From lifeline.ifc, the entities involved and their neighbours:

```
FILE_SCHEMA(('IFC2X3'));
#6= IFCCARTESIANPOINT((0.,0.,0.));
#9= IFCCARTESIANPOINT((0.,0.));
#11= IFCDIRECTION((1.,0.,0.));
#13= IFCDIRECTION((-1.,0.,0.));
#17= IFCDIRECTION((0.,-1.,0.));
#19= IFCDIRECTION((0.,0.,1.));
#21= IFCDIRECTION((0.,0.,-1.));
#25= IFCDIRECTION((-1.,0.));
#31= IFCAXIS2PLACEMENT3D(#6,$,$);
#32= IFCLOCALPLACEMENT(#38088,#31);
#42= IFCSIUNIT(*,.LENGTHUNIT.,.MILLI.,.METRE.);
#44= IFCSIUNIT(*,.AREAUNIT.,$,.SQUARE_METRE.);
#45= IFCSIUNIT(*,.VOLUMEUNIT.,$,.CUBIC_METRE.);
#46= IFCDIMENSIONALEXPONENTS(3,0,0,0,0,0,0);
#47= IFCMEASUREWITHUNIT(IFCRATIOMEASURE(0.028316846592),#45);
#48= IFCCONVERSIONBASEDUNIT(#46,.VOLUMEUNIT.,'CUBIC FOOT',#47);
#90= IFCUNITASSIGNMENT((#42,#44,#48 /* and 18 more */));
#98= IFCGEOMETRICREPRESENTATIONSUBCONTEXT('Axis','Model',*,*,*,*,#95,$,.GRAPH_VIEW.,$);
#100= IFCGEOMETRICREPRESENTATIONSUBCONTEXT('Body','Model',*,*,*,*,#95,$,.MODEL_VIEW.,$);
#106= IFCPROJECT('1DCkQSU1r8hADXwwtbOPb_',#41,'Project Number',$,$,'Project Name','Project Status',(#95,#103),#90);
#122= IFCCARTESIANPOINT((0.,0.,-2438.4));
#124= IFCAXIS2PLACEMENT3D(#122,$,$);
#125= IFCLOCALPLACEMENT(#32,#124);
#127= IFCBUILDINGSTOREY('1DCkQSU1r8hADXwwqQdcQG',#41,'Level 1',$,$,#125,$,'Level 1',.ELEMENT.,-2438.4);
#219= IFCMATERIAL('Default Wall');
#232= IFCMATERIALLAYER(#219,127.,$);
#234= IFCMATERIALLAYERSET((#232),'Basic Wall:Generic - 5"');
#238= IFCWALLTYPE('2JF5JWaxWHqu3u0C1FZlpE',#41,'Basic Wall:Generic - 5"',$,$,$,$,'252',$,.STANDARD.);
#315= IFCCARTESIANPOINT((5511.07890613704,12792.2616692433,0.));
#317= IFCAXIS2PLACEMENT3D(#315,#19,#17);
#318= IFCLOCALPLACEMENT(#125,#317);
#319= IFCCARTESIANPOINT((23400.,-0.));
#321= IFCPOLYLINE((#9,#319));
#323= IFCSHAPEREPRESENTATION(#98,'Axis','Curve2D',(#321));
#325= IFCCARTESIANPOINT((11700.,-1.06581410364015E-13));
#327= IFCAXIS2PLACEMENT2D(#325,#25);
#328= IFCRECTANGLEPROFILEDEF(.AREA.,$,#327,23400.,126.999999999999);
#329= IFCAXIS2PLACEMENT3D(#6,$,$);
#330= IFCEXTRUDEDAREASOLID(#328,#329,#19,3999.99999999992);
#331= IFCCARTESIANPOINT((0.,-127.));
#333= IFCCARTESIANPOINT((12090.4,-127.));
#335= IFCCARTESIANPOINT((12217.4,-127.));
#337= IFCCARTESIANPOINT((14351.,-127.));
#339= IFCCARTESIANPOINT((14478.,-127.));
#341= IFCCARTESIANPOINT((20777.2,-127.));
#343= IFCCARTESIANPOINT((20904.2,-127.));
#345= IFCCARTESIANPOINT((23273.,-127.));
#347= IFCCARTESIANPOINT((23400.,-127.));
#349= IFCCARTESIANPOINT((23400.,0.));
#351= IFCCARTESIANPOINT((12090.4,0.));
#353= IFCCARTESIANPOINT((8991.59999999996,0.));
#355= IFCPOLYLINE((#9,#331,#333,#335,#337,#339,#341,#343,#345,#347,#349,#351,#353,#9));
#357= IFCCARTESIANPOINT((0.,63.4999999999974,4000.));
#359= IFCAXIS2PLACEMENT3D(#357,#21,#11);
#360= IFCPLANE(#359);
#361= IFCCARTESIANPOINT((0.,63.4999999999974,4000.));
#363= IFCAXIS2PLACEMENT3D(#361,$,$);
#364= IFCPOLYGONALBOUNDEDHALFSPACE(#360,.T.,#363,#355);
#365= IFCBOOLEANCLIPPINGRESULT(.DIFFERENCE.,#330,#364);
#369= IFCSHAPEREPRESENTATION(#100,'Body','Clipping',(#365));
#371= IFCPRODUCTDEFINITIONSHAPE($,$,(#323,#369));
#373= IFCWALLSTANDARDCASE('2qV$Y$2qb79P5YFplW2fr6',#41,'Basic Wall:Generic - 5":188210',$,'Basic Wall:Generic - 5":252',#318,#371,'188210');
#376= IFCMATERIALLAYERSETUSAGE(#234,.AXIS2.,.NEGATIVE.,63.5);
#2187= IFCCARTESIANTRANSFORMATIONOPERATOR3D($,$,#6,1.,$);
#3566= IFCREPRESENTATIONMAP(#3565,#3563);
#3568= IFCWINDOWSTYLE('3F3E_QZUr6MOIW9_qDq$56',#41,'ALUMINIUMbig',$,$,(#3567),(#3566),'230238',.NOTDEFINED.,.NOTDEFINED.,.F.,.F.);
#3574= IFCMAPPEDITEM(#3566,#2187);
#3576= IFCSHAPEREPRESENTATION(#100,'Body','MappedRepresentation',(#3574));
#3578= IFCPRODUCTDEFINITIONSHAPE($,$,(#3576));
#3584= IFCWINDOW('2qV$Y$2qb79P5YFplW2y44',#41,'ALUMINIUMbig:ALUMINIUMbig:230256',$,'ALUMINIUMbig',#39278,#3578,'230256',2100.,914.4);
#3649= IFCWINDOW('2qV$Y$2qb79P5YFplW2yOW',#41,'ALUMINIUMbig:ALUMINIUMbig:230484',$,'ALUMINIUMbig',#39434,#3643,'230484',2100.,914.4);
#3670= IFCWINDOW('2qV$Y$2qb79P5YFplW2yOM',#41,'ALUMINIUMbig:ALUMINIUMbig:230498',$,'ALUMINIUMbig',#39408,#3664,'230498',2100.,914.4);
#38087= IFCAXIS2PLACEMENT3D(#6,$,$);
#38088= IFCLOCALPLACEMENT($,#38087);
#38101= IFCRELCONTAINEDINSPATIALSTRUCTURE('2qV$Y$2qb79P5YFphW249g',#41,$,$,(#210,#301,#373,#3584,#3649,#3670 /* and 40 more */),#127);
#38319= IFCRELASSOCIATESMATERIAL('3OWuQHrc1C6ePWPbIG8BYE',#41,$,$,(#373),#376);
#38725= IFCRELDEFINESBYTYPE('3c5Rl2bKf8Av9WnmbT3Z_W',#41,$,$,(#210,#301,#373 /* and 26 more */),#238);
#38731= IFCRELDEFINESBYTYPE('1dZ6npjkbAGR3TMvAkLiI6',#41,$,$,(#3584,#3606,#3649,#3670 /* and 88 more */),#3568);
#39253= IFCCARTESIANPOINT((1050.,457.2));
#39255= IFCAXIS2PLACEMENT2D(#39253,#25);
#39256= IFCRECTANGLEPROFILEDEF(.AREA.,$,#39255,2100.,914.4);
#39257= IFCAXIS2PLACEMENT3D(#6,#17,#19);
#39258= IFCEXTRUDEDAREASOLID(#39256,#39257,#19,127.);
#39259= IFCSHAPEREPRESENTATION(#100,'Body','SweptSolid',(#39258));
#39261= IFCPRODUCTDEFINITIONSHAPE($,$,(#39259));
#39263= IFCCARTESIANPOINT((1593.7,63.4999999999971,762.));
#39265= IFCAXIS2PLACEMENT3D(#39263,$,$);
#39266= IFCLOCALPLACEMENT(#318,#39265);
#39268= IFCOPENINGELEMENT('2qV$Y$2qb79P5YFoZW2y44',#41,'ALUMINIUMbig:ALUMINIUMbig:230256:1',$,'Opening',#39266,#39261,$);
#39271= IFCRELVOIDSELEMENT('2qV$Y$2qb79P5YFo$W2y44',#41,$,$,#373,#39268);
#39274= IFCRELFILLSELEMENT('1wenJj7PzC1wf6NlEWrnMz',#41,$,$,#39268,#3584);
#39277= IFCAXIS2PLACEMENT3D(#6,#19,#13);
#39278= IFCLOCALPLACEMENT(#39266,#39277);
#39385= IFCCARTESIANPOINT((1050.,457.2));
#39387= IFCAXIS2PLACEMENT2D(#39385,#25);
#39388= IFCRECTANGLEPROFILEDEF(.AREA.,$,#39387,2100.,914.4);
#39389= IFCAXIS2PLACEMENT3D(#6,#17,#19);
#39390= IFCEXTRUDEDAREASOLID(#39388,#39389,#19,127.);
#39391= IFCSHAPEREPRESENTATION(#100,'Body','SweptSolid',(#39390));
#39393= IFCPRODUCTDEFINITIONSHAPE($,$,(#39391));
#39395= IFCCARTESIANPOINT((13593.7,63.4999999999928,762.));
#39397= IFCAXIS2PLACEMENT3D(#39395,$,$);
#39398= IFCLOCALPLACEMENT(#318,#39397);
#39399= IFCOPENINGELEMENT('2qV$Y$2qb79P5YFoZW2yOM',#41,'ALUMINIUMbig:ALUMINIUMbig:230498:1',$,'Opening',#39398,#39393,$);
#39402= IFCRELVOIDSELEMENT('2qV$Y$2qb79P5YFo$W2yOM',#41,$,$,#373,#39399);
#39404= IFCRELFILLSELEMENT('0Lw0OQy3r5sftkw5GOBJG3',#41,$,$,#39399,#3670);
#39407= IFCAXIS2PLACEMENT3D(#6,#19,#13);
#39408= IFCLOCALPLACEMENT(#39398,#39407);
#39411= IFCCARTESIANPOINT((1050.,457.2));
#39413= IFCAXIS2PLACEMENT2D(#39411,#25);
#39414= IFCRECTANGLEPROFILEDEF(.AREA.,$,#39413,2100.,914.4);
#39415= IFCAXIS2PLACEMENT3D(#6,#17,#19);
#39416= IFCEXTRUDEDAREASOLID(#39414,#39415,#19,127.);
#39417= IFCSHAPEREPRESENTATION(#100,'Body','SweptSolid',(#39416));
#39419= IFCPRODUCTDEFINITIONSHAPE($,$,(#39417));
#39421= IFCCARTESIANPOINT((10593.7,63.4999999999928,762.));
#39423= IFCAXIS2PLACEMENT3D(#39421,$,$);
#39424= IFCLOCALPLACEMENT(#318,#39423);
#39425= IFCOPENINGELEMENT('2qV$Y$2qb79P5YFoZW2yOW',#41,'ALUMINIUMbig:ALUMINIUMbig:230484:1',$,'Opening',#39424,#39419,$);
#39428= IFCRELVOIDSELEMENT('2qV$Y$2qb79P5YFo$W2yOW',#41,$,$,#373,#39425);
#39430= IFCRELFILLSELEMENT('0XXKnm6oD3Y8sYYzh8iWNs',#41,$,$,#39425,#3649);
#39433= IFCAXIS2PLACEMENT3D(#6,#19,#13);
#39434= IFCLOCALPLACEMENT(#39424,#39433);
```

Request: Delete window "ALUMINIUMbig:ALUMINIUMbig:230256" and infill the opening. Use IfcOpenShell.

```python
import ifcopenshell
import ifcopenshell.api.feature
import ifcopenshell.api.root
import ifcopenshell.geom
import ifcopenshell.util.shape

model = ifcopenshell.open("lifeline.ifc")
settings = ifcopenshell.geom.settings()


def volume(element):
    """Net volume in cubic metres, openings subtracted."""
    shape = ifcopenshell.geom.create_shape(settings, element)
    return ifcopenshell.util.shape.get_volume(shape.geometry)


window = model.by_guid("2qV$Y$2qb79P5YFplW2y44")
opening = window.FillsVoids[0].RelatingOpeningElement
wall = opening.VoidsElements[0].RelatingBuildingElement
before = volume(wall)

ifcopenshell.api.root.remove_product(model, product=window)
ifcopenshell.api.feature.remove_feature(model, feature=opening)

after = volume(wall)

print(f"wall volume {before:.3f} -> {after:.3f} m3")

model.write("lifeline_rev.ifc")
```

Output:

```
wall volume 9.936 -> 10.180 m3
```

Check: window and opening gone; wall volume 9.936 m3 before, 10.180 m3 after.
